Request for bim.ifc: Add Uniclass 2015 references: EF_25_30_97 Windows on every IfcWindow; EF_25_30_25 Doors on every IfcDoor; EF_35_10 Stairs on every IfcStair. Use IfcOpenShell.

First a look at what the model holds.

```python
import ifcopenshell

model = ifcopenshell.open("bim.ifc")
print(model.schema)
print("classifications:", [c.Name for c in model.by_type("IfcClassification")])
for ifc_class in ("IfcDoor", "IfcRoof", "IfcStair", "IfcWall", "IfcWindow"):
    print(ifc_class, len(model.by_type(ifc_class)))
```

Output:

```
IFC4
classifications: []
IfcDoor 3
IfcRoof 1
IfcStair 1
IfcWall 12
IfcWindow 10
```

```python
import ifcopenshell
import ifcopenshell.api.classification

model = ifcopenshell.open("bim.ifc")

system = ifcopenshell.api.classification.add_classification(model, classification="Uniclass 2015")

codes = {
    "IfcWindow": ("EF_25_30_97", "Windows"),
    "IfcDoor": ("EF_25_30_25", "Doors"),
    "IfcStair": ("EF_35_10", "Stairs"),
}
for ifc_class, (code, name) in codes.items():
    products = model.by_type(ifc_class)
    ifcopenshell.api.classification.add_reference(
        model, products=products, classification=system, identification=code, name=name
    )
    print(code, len(products))

model.write("bim_rev.ifc")
```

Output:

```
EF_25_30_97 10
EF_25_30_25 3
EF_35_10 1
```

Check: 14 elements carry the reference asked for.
